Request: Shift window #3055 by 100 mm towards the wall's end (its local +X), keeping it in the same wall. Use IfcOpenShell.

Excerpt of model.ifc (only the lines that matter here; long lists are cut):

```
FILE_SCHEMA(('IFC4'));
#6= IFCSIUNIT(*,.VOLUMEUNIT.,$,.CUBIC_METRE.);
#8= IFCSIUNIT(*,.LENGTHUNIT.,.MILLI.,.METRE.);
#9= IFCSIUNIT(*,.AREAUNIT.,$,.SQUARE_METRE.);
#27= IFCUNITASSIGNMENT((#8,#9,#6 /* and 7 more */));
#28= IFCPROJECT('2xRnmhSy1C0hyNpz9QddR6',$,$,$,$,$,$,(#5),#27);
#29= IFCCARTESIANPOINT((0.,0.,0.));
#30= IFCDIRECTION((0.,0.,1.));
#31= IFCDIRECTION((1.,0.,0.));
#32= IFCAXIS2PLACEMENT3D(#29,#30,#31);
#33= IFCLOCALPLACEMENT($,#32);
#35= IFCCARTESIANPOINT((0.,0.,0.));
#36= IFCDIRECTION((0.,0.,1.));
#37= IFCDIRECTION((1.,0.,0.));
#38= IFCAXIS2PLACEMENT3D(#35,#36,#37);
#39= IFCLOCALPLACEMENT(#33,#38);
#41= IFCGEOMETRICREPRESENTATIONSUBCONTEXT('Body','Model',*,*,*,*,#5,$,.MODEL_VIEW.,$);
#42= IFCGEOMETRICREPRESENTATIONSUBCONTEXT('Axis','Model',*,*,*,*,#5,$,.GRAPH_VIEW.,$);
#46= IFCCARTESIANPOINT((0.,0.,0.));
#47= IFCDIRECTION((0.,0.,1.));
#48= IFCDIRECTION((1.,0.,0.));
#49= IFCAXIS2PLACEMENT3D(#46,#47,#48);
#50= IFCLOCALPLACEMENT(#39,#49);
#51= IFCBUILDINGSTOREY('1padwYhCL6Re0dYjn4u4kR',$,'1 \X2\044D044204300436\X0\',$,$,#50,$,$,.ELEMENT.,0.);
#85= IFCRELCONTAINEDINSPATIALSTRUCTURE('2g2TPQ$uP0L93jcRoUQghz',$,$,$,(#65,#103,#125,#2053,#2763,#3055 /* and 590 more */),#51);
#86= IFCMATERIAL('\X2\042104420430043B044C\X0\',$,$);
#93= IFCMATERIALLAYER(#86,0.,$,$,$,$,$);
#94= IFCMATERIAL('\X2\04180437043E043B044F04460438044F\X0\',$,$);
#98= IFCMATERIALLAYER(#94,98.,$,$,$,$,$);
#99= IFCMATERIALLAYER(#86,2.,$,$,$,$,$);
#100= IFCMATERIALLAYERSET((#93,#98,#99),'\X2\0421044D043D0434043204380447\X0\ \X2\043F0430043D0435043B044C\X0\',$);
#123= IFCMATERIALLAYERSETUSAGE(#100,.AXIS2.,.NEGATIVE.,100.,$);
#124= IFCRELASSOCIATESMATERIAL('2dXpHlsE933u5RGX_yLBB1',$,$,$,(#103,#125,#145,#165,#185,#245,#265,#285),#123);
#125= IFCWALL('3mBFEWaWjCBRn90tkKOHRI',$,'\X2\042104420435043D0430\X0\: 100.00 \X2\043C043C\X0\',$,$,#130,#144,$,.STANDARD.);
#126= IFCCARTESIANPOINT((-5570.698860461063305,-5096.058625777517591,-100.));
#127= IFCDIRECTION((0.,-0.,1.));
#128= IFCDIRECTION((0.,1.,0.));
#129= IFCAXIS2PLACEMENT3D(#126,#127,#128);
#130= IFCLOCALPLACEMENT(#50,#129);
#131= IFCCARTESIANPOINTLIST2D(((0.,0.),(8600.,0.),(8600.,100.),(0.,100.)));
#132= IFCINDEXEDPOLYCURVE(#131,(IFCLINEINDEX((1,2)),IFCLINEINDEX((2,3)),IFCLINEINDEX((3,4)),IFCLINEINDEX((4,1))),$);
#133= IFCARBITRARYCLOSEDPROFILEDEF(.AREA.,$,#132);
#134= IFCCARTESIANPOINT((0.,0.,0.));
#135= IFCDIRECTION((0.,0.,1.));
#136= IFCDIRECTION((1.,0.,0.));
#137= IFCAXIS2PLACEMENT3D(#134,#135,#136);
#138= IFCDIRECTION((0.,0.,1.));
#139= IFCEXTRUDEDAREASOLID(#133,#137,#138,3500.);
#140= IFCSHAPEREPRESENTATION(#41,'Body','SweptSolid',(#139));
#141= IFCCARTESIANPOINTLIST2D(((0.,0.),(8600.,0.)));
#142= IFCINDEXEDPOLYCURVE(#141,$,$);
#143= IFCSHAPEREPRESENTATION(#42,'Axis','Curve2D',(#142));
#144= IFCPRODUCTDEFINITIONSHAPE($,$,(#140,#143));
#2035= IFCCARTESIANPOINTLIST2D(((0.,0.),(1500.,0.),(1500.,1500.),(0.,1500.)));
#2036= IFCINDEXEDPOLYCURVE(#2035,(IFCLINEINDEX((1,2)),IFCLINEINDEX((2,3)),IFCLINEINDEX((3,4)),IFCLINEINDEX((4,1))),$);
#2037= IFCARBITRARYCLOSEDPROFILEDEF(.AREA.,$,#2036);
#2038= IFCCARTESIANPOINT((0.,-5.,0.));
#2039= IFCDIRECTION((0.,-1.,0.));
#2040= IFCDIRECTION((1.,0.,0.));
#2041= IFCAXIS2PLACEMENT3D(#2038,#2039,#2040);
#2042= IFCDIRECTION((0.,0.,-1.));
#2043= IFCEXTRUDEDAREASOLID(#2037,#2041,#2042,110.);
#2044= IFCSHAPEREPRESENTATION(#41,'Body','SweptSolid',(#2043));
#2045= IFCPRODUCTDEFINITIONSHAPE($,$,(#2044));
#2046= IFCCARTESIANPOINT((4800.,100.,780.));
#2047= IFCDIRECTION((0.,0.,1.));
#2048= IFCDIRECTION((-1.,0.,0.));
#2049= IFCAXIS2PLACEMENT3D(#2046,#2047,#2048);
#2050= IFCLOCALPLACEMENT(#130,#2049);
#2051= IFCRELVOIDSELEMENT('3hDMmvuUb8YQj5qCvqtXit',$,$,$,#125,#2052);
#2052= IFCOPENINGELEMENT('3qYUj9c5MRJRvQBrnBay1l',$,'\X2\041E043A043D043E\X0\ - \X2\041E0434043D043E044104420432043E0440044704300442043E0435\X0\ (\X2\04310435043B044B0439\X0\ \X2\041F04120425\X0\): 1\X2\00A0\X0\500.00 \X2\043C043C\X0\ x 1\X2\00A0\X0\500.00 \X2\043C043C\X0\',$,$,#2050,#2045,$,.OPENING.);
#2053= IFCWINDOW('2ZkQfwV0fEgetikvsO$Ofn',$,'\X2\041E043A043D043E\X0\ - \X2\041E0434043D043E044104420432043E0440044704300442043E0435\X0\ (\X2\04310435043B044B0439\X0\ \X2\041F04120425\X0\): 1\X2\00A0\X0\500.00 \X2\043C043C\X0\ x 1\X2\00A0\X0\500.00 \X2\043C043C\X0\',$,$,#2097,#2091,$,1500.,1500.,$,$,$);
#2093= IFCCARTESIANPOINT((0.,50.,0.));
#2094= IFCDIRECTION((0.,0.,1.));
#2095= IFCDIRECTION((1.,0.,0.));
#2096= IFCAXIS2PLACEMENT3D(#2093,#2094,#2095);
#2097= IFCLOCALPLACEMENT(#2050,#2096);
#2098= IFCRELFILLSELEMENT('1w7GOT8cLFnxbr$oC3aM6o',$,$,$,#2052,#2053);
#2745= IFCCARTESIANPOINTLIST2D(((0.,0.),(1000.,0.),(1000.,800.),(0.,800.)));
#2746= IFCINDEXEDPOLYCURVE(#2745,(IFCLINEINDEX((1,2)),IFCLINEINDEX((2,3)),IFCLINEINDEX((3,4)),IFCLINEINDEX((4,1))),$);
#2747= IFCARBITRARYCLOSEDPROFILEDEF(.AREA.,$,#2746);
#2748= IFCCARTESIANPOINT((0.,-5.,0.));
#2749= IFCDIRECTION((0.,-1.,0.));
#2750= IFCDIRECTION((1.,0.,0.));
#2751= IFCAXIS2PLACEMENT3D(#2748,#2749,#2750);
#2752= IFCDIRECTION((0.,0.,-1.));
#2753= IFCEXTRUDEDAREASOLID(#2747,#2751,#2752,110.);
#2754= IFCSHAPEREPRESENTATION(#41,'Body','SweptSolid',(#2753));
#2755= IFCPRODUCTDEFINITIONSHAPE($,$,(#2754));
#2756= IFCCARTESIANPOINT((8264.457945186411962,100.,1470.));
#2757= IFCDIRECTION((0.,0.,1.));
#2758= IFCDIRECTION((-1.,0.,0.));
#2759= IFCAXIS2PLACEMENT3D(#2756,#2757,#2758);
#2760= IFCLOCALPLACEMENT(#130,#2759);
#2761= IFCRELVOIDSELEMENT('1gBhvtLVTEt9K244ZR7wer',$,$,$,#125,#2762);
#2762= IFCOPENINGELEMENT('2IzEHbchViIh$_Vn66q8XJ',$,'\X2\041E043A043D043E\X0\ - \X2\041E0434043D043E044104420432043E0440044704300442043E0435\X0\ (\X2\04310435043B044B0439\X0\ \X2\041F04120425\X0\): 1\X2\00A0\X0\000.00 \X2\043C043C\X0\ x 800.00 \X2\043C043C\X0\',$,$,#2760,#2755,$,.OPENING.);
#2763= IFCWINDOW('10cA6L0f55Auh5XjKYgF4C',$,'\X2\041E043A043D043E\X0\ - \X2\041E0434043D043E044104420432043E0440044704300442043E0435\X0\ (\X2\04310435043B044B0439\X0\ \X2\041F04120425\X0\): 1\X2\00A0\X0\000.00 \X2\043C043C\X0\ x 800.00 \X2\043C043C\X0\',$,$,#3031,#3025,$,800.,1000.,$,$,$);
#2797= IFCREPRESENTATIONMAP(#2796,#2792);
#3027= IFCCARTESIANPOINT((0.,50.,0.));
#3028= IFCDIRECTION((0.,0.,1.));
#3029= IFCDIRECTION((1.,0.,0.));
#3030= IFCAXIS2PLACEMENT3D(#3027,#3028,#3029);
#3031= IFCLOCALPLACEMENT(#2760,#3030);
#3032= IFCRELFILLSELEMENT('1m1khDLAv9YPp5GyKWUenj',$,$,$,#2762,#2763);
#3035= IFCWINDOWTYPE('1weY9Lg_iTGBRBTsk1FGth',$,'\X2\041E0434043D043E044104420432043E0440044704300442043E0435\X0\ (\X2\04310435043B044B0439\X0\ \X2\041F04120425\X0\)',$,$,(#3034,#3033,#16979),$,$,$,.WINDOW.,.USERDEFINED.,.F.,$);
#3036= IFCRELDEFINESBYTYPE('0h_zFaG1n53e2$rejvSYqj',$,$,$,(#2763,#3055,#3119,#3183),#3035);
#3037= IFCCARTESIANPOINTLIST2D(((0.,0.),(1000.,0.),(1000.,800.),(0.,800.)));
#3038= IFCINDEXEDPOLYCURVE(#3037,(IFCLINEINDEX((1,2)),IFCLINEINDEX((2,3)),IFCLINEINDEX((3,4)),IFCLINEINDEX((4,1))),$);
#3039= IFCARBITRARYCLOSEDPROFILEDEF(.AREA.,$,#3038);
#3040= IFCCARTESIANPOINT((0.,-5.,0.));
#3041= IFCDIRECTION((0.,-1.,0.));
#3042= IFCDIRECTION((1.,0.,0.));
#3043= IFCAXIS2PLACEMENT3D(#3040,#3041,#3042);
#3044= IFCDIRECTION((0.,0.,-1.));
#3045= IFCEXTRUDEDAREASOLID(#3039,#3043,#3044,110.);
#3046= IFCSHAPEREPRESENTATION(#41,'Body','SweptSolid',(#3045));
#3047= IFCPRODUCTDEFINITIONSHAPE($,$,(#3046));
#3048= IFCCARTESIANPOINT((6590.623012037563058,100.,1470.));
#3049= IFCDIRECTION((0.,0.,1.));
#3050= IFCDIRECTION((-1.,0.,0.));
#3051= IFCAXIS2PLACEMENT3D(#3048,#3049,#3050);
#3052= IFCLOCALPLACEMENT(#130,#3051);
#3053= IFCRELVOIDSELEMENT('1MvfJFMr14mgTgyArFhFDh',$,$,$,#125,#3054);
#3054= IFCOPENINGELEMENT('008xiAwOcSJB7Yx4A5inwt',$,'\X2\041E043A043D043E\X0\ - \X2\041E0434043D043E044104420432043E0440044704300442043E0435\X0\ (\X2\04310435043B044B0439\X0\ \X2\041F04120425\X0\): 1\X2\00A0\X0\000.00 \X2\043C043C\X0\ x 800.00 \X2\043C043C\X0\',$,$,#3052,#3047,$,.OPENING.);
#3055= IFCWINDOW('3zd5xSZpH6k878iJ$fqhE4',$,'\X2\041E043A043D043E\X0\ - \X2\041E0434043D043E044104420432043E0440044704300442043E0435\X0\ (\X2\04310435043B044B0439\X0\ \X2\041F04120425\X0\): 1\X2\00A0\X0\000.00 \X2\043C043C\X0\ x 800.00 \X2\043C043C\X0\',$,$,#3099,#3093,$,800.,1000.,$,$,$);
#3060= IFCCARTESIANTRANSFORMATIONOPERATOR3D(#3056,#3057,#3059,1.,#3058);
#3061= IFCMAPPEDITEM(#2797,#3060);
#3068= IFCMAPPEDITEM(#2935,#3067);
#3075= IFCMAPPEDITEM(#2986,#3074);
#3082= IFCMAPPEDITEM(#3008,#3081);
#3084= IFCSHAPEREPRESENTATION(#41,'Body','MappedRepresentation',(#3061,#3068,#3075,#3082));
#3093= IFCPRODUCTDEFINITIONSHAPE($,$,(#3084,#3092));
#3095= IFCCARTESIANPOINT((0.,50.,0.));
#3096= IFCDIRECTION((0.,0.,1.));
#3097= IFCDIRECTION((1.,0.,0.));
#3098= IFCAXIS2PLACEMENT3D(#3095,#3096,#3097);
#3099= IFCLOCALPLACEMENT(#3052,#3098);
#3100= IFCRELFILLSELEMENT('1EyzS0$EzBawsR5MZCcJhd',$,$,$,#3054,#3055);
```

```python
import ifcopenshell
import ifcopenshell.api.geometry
import ifcopenshell.util.placement

model = ifcopenshell.open("model.ifc")

window = model.by_guid("3zd5xSZpH6k878iJ$fqhE4")
opening = window.FillsVoids[0].RelatingOpeningElement
wall = opening.VoidsElements[0].RelatingBuildingElement

wall_matrix = ifcopenshell.util.placement.get_local_placement(wall.ObjectPlacement)
shift = wall_matrix[:3, 0] * 100.0
before = ifcopenshell.util.placement.get_local_placement(window.ObjectPlacement)[:3, 3].copy()

# The window is placed relative to its opening, so it follows when the opening moves.
matrix = ifcopenshell.util.placement.get_local_placement(opening.ObjectPlacement)
matrix[:3, 3] += shift
ifcopenshell.api.geometry.edit_object_placement(
    model, product=opening, matrix=matrix, is_si=False, should_transform_children=True
)

after = ifcopenshell.util.placement.get_local_placement(window.ObjectPlacement)[:3, 3]
print("window moved by", (after - before).round(3) + 0.0)

model.write("model-out.ifc")
```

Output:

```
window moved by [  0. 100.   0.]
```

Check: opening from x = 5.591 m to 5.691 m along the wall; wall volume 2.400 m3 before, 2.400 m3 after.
